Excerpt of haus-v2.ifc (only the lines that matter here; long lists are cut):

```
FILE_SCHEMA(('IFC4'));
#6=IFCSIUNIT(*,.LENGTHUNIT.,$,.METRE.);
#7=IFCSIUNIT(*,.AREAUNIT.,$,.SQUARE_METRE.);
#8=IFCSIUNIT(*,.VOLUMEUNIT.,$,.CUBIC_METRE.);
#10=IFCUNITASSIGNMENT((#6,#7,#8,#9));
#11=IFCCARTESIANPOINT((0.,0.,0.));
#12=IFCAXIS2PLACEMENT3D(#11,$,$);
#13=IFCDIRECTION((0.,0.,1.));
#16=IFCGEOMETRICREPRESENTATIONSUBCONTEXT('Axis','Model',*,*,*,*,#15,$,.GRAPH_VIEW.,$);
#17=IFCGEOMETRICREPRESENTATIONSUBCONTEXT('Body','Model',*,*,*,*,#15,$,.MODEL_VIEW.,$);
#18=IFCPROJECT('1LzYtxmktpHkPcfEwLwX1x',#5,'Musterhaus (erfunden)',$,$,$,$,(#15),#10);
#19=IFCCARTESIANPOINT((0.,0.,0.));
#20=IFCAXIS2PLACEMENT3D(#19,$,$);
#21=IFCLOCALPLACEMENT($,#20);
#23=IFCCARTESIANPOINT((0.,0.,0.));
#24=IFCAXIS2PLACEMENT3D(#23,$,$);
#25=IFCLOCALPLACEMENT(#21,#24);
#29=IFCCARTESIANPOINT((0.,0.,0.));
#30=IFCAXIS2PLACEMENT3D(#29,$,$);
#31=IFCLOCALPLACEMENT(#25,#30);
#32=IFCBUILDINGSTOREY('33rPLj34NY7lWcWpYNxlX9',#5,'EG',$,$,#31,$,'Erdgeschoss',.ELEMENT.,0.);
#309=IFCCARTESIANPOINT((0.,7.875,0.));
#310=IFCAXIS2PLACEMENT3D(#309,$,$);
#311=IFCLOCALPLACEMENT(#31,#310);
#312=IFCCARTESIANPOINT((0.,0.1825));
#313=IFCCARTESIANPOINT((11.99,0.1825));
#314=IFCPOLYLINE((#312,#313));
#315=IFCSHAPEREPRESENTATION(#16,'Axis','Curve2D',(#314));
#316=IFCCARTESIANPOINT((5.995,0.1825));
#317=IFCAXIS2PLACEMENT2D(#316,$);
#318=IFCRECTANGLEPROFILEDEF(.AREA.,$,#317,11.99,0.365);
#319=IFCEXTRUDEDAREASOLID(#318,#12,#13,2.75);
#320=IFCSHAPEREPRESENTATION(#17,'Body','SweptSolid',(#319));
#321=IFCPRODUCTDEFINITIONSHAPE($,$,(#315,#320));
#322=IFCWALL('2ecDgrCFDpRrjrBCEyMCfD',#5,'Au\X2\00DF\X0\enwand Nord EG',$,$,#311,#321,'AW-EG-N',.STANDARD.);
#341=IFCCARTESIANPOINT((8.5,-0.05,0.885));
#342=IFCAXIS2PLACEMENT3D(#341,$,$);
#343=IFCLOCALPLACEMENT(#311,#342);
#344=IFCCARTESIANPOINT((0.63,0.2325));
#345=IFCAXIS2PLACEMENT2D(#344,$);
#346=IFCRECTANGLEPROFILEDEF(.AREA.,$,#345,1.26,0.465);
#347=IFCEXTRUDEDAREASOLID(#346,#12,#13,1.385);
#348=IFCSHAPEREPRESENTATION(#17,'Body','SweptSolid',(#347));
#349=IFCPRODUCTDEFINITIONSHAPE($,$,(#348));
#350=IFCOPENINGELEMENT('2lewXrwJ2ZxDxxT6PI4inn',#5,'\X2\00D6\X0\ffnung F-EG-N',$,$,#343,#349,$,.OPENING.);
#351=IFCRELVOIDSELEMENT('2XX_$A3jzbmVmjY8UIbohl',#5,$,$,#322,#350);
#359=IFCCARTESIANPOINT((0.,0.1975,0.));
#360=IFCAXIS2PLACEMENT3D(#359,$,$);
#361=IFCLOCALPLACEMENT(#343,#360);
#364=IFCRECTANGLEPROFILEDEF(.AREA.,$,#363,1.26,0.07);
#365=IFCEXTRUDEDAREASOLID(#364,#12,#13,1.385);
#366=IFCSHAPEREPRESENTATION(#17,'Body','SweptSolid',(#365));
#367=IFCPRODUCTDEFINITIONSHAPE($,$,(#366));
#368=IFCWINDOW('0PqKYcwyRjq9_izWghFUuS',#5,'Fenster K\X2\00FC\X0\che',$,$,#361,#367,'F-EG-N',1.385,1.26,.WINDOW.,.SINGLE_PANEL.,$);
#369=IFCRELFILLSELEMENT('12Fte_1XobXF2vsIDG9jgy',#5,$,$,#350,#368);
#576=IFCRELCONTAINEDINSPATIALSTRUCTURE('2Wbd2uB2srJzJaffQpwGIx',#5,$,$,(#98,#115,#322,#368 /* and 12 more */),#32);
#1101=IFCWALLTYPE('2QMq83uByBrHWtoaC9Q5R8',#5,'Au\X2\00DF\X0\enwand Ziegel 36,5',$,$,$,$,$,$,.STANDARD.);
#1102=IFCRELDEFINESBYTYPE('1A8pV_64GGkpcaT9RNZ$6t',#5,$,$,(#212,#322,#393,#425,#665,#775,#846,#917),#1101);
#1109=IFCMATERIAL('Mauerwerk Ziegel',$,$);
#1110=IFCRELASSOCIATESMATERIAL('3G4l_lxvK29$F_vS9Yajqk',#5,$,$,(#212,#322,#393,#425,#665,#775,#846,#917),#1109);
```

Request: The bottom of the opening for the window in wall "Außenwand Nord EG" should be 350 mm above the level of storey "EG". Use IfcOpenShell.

```python
import numpy as np
import ifcopenshell
import ifcopenshell.api.geometry
import ifcopenshell.geom
import ifcopenshell.util.element
import ifcopenshell.util.placement
import ifcopenshell.util.shape
import ifcopenshell.util.unit

model = ifcopenshell.open("haus-v2.ifc")
unit_scale = ifcopenshell.util.unit.calculate_unit_scale(model)

window = model.by_id(368)
opening = window.FillsVoids[0].RelatingOpeningElement
storey = ifcopenshell.util.element.get_container(window, ifc_class="IfcBuildingStorey")
level = ifcopenshell.util.placement.get_local_placement(storey.ObjectPlacement)[2, 3]

# The opening's origin need not be at the sill, so measure its lowest point.
shape = ifcopenshell.geom.create_shape(ifcopenshell.geom.settings(), opening)
bottom = ifcopenshell.util.shape.get_shape_bottom_elevation(shape, shape.geometry) / unit_scale
dz = level + 0.35 / unit_scale - bottom

shift = np.array([0.0, 0.0, dz])
# The window is placed relative to its opening, so it follows when the opening moves.
matrix = ifcopenshell.util.placement.get_local_placement(opening.ObjectPlacement)
matrix[:3, 3] += shift
ifcopenshell.api.geometry.edit_object_placement(
    model, product=opening, matrix=matrix, is_si=False, should_transform_children=True
)

print(f"moved by {dz * unit_scale:+.3f} m")

model.write("haus-v2_v2.ifc")
```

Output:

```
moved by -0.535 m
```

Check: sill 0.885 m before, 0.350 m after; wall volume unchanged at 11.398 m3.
